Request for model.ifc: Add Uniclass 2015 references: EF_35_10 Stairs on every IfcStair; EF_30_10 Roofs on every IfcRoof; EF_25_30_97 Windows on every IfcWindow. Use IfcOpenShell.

First a look at what the model holds.

```python
import ifcopenshell

model = ifcopenshell.open("model.ifc")
print(model.schema)
print("classifications:", [c.Name for c in model.by_type("IfcClassification")])
for ifc_class in ("IfcDoor", "IfcRoof", "IfcStair", "IfcWall", "IfcWindow"):
    print(ifc_class, len(model.by_type(ifc_class)))
```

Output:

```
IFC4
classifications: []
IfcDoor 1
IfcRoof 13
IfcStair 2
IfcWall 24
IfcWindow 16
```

```python
import ifcopenshell
import ifcopenshell.api.classification

model = ifcopenshell.open("model.ifc")

system = ifcopenshell.api.classification.add_classification(model, classification="Uniclass 2015")

codes = {
    "IfcStair": ("EF_35_10", "Stairs"),
    "IfcRoof": ("EF_30_10", "Roofs"),
    "IfcWindow": ("EF_25_30_97", "Windows"),
}
for ifc_class, (code, name) in codes.items():
    products = model.by_type(ifc_class)
    ifcopenshell.api.classification.add_reference(
        model, products=products, classification=system, identification=code, name=name
    )
    print(code, len(products))

model.write("model-out.ifc")
```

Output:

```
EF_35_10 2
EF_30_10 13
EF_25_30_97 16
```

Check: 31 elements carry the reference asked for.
